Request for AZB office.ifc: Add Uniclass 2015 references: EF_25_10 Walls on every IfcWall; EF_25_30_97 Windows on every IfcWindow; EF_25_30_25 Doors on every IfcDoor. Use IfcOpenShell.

First a look at what the model holds.

```python
import ifcopenshell

model = ifcopenshell.open("AZB office.ifc")
print(model.schema)
print("classifications:", [c.Name for c in model.by_type("IfcClassification")])
for ifc_class in ("IfcDoor", "IfcRoof", "IfcStair", "IfcWall", "IfcWindow"):
    print(ifc_class, len(model.by_type(ifc_class)))
```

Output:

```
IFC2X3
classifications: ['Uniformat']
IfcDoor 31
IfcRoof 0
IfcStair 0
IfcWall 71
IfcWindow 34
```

```python
import ifcopenshell
import ifcopenshell.api.classification

model = ifcopenshell.open("AZB office.ifc")

# IFC2X3 requires Source and Edition and has no link from the project to the system.
system = model.create_entity("IfcClassification", Source="NBS", Edition="2015", Name="Uniclass 2015")

codes = {
    "IfcWall": ("EF_25_10", "Walls"),
    "IfcWindow": ("EF_25_30_97", "Windows"),
    "IfcDoor": ("EF_25_30_25", "Doors"),
}
for ifc_class, (code, name) in codes.items():
    products = model.by_type(ifc_class)
    ifcopenshell.api.classification.add_reference(
        model, products=products, classification=system, identification=code, name=name
    )
    print(code, len(products))

model.write("AZB office_rev.ifc")
```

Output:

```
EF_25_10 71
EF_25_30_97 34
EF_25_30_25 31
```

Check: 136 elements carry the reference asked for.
